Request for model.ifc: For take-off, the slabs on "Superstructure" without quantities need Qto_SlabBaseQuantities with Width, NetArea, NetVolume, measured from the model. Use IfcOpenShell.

First a look at what the model holds.

```python
import ifcopenshell
import ifcopenshell.util.element
import ifcopenshell.util.unit

model = ifcopenshell.open("model.ifc")
print(model.schema)
for unit_type in ("LENGTHUNIT", "AREAUNIT", "VOLUMEUNIT"):
    print(unit_type, ifcopenshell.util.unit.calculate_unit_scale(model, unit_type))
storey = next(s for s in model.by_type("IfcBuildingStorey") if s.Name == "Superstructure")
slabs = [e for e in ifcopenshell.util.element.get_decomposition(storey) if e.is_a("IfcSlab")]
for e in sorted(slabs, key=lambda e: e.id()):
    print(e.id(), e.is_a(), e.Name, list(ifcopenshell.util.element.get_psets(e, qtos_only=True)), sep=" | ")
```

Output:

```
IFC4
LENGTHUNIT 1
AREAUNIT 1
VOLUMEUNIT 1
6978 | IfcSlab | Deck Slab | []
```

```python
import ifcopenshell
import ifcopenshell.api.pset
import ifcopenshell.geom
import ifcopenshell.util.element
import ifcopenshell.util.shape
import ifcopenshell.util.unit

model = ifcopenshell.open("model.ifc")
unit_scale = ifcopenshell.util.unit.calculate_unit_scale(model)
area_scale = ifcopenshell.util.unit.calculate_unit_scale(model, "AREAUNIT")
volume_scale = ifcopenshell.util.unit.calculate_unit_scale(model, "VOLUMEUNIT")
settings = ifcopenshell.geom.settings()

storey = next(s for s in model.by_type("IfcBuildingStorey") if s.Name == "Superstructure")
slabs = [e for e in ifcopenshell.util.element.get_decomposition(storey) if e.is_a("IfcSlab")]

for e in sorted(slabs, key=lambda e: e.id()):
    if ifcopenshell.util.element.get_psets(e, qtos_only=True, should_inherit=False):
        continue
    # Geometry comes back in metres, in the element's own axes.
    shape = ifcopenshell.geom.create_shape(settings, e)
    values = {
        "Width": ifcopenshell.util.shape.get_z(shape.geometry) / unit_scale,
        "NetArea": ifcopenshell.util.shape.get_footprint_area(shape.geometry) / area_scale,
        "NetVolume": ifcopenshell.util.shape.get_volume(shape.geometry) / volume_scale,
    }
    qto = ifcopenshell.api.pset.add_qto(model, product=e, name="Qto_SlabBaseQuantities")
    ifcopenshell.api.pset.edit_qto(model, qto=qto, properties=values)
    print(e.id(), {k: round(v, 3) for k, v in values.items()})

model.write("model-out.ifc")
```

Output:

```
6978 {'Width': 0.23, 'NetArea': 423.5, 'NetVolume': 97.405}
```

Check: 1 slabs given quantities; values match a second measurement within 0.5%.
